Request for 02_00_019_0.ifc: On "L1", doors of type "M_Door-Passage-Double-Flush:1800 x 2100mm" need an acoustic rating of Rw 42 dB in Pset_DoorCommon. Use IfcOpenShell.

First a look at what the model holds.

```python
import ifcopenshell
import ifcopenshell.util.element

model = ifcopenshell.open("02_00_019_0.ifc")
print(model.schema)
storey = next(s for s in model.by_type("IfcBuildingStorey") if s.Name == "L1")
doors = [e for e in ifcopenshell.util.element.get_decomposition(storey) if e.is_a("IfcDoor")]
seen = {}
for e in doors:
    element_type = ifcopenshell.util.element.get_type(e)
    key = (element_type.Name if element_type != e and element_type else None, ifcopenshell.util.element.get_pset(e, "Pset_DoorCommon", "AcousticRating"))
    seen[key] = seen.get(key, 0) + 1
for (name, value), count in sorted(seen.items(), key=str):
    print(count, "x", name, "|", value)
```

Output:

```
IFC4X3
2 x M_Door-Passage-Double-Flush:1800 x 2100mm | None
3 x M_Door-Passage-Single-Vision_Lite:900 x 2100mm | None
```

```python
import ifcopenshell
import ifcopenshell.api.pset
import ifcopenshell.util.element

model = ifcopenshell.open("02_00_019_0.ifc")

storey = next(s for s in model.by_type("IfcBuildingStorey") if s.Name == "L1")
doors = [e for e in ifcopenshell.util.element.get_decomposition(storey) if e.is_a("IfcDoor")]

count = 0
for e in doors:
    element_type = ifcopenshell.util.element.get_type(e)
    if element_type in (None, e) or element_type.Name != "M_Door-Passage-Double-Flush:1800 x 2100mm":
        continue
    # add_pset returns the element's existing set when there is one.
    pset = ifcopenshell.api.pset.add_pset(model, product=e, name="Pset_DoorCommon")
    ifcopenshell.api.pset.edit_pset(model, pset=pset, properties={"AcousticRating": "Rw 42 dB"})
    count += 1

print(count, "doors updated")

model.write("02_00_019_0-out.ifc")
```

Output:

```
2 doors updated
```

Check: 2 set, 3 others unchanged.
